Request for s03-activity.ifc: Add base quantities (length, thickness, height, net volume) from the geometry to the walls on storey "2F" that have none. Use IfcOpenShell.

First a look at what the model holds.

```python
import ifcopenshell
import ifcopenshell.util.element
import ifcopenshell.util.unit

model = ifcopenshell.open("s03-activity.ifc")
print(model.schema)
for unit_type in ("LENGTHUNIT", "AREAUNIT", "VOLUMEUNIT"):
    print(unit_type, ifcopenshell.util.unit.calculate_unit_scale(model, unit_type))
storey = next(s for s in model.by_type("IfcBuildingStorey") if s.Name == "2F")
walls = [e for e in ifcopenshell.util.element.get_decomposition(storey) if e.is_a("IfcWall")]
for e in sorted(walls, key=lambda e: e.id()):
    print(e.id(), e.is_a(), e.Name, list(ifcopenshell.util.element.get_psets(e, qtos_only=True)), sep=" | ")
```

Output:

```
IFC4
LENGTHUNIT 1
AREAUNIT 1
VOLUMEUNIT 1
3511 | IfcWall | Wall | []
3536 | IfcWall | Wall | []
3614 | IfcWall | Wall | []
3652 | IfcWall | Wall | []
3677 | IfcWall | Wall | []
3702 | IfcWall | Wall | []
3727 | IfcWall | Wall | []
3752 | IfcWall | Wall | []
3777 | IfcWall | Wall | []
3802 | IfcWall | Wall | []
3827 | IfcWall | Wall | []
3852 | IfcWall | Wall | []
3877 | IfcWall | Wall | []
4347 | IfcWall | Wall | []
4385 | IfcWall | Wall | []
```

```python
import ifcopenshell
import ifcopenshell.api.pset
import ifcopenshell.geom
import ifcopenshell.util.element
import ifcopenshell.util.shape
import ifcopenshell.util.unit

model = ifcopenshell.open("s03-activity.ifc")
unit_scale = ifcopenshell.util.unit.calculate_unit_scale(model)
volume_scale = ifcopenshell.util.unit.calculate_unit_scale(model, "VOLUMEUNIT")
settings = ifcopenshell.geom.settings()

storey = next(s for s in model.by_type("IfcBuildingStorey") if s.Name == "2F")
walls = [e for e in ifcopenshell.util.element.get_decomposition(storey) if e.is_a("IfcWall")]

for e in sorted(walls, key=lambda e: e.id()):
    if ifcopenshell.util.element.get_psets(e, qtos_only=True, should_inherit=False):
        continue
    # Geometry comes back in metres, in the element's own axes.
    shape = ifcopenshell.geom.create_shape(settings, e)
    values = {
        "Length": ifcopenshell.util.shape.get_x(shape.geometry) / unit_scale,
        "Width": ifcopenshell.util.shape.get_y(shape.geometry) / unit_scale,
        "Height": ifcopenshell.util.shape.get_z(shape.geometry) / unit_scale,
        "NetVolume": ifcopenshell.util.shape.get_volume(shape.geometry) / volume_scale,
    }
    qto = ifcopenshell.api.pset.add_qto(model, product=e, name="Qto_WallBaseQuantities")
    ifcopenshell.api.pset.edit_qto(model, qto=qto, properties=values)
    print(e.id(), {k: round(v, 3) for k, v in values.items()})

model.write("s03-activity_rev.ifc")
```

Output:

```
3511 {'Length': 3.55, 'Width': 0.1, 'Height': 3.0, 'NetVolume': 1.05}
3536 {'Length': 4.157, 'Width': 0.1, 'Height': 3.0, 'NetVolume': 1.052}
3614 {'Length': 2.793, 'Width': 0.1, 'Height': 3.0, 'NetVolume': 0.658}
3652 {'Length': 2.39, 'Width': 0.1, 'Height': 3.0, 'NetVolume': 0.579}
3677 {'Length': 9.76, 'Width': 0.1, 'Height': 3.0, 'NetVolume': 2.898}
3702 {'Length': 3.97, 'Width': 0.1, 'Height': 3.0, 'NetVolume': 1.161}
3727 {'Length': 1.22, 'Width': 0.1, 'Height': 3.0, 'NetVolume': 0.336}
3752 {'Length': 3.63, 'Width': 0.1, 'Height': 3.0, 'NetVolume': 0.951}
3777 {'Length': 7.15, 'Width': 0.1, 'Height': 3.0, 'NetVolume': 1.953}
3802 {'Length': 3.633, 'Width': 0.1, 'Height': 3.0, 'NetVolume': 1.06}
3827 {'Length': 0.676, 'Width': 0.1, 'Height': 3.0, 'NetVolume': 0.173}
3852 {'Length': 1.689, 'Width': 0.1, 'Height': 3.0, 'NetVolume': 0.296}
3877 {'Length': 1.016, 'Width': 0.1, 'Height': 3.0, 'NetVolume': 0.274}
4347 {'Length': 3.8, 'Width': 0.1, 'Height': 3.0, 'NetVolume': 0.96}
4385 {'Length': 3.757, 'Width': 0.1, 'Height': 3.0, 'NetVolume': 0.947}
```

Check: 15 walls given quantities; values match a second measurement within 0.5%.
